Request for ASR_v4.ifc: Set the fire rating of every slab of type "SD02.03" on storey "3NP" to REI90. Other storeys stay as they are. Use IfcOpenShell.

First a look at what the model holds.

```python
import ifcopenshell
import ifcopenshell.util.element

model = ifcopenshell.open("ASR_v4.ifc")
print(model.schema)
storey = next(s for s in model.by_type("IfcBuildingStorey") if s.Name == "3NP")
slabs = [e for e in ifcopenshell.util.element.get_decomposition(storey) if e.is_a("IfcSlab")]
seen = {}
for e in slabs:
    element_type = ifcopenshell.util.element.get_type(e)
    key = (element_type.Name if element_type != e and element_type else None, ifcopenshell.util.element.get_pset(e, "Pset_SlabCommon", "FireRating"))
    seen[key] = seen.get(key, 0) + 1
for (name, value), count in sorted(seen.items(), key=str):
    print(count, "x", name, "|", value)
```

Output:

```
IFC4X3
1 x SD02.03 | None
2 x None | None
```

```python
import ifcopenshell
import ifcopenshell.api.pset
import ifcopenshell.util.element

model = ifcopenshell.open("ASR_v4.ifc")

storey = next(s for s in model.by_type("IfcBuildingStorey") if s.Name == "3NP")
slabs = [e for e in ifcopenshell.util.element.get_decomposition(storey) if e.is_a("IfcSlab")]

count = 0
for e in slabs:
    element_type = ifcopenshell.util.element.get_type(e)
    if element_type in (None, e) or element_type.Name != "SD02.03":
        continue
    # add_pset returns the element's existing set when there is one.
    pset = ifcopenshell.api.pset.add_pset(model, product=e, name="Pset_SlabCommon")
    ifcopenshell.api.pset.edit_pset(model, pset=pset, properties={"FireRating": "REI90"})
    count += 1

print(count, "slabs updated")

model.write("ASR_v4-out.ifc")
```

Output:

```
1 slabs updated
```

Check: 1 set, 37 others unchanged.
